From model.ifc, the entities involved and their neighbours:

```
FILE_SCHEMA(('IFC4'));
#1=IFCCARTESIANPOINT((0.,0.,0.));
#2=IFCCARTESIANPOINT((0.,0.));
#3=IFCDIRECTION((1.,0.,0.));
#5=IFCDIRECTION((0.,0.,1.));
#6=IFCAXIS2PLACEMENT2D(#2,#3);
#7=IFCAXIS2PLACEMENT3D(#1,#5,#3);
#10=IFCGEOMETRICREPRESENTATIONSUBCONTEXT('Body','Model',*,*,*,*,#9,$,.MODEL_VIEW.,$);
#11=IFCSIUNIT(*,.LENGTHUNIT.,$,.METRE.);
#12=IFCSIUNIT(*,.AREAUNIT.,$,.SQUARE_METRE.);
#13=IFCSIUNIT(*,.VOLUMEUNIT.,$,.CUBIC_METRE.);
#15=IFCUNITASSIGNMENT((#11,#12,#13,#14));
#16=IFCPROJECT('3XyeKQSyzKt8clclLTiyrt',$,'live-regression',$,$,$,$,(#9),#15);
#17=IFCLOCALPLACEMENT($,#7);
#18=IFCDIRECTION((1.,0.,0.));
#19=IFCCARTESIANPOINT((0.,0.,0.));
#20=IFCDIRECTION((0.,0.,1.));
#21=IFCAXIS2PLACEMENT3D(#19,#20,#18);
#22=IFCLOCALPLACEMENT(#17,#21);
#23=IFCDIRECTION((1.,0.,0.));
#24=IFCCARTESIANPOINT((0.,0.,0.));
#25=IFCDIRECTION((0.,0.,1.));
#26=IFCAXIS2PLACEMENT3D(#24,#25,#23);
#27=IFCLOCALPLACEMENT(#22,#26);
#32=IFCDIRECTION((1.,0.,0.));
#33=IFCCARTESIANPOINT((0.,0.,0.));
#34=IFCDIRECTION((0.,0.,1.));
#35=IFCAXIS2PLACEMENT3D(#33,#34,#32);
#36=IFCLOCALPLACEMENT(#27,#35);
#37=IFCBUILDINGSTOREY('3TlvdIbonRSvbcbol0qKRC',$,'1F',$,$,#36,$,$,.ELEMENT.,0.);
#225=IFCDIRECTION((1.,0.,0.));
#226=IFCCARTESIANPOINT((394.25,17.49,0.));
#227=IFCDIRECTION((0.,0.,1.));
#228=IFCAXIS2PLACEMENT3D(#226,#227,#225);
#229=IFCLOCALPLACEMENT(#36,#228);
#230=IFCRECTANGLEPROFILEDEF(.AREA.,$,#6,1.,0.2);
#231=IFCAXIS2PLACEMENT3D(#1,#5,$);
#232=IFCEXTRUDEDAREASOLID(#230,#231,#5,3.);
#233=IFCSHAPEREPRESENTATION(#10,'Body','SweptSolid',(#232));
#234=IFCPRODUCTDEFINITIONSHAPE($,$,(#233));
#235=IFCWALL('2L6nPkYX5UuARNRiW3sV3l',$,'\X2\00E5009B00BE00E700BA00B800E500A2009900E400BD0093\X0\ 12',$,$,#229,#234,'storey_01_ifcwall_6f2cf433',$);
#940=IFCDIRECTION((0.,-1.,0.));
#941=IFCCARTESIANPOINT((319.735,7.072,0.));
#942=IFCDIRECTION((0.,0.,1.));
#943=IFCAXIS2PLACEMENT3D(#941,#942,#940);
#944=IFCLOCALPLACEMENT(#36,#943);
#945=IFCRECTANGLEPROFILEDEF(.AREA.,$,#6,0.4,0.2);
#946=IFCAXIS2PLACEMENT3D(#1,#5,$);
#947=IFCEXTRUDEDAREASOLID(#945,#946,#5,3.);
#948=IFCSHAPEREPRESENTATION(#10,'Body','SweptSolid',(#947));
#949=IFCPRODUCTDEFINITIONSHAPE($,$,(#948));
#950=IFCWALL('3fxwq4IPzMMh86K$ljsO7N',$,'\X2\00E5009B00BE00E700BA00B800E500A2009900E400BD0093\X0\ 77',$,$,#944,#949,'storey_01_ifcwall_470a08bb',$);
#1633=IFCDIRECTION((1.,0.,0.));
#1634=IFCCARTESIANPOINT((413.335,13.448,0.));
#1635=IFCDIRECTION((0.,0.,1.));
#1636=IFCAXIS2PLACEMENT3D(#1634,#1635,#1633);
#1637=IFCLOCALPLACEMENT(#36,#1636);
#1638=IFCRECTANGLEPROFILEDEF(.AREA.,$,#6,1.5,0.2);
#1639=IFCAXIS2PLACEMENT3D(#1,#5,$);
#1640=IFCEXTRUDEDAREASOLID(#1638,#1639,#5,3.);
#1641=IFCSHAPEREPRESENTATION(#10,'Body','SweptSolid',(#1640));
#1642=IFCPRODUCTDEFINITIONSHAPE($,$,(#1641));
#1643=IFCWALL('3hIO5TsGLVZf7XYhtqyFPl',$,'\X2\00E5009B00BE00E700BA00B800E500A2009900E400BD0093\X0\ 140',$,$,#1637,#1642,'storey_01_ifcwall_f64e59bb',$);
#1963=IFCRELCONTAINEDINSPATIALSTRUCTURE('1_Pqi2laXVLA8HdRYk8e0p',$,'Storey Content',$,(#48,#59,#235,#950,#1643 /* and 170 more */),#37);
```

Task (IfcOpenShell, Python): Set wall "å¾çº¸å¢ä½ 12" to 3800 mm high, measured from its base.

```python
import ifcopenshell
import ifcopenshell.geom
import ifcopenshell.util.representation
import ifcopenshell.util.shape

model = ifcopenshell.open("model.ifc")
settings = ifcopenshell.geom.settings()


def volume(element):
    """Net volume in cubic metres, openings subtracted."""
    shape = ifcopenshell.geom.create_shape(settings, element)
    return ifcopenshell.util.shape.get_volume(shape.geometry)


wall = model.by_guid("2L6nPkYX5UuARNRiW3sV3l")
before = volume(wall)

body = ifcopenshell.util.representation.get_representation(wall, "Model", "Body")
solid = body.Items[0]
old_height = solid.Depth
solid.Depth = 3.8
after = volume(wall)

print(f"height {old_height:g} -> {solid.Depth:g}, volume {before:.3f} -> {after:.3f} m3")

model.write("model-out.ifc")
```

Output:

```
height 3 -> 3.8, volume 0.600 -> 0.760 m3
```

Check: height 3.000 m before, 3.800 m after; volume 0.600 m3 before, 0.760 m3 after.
